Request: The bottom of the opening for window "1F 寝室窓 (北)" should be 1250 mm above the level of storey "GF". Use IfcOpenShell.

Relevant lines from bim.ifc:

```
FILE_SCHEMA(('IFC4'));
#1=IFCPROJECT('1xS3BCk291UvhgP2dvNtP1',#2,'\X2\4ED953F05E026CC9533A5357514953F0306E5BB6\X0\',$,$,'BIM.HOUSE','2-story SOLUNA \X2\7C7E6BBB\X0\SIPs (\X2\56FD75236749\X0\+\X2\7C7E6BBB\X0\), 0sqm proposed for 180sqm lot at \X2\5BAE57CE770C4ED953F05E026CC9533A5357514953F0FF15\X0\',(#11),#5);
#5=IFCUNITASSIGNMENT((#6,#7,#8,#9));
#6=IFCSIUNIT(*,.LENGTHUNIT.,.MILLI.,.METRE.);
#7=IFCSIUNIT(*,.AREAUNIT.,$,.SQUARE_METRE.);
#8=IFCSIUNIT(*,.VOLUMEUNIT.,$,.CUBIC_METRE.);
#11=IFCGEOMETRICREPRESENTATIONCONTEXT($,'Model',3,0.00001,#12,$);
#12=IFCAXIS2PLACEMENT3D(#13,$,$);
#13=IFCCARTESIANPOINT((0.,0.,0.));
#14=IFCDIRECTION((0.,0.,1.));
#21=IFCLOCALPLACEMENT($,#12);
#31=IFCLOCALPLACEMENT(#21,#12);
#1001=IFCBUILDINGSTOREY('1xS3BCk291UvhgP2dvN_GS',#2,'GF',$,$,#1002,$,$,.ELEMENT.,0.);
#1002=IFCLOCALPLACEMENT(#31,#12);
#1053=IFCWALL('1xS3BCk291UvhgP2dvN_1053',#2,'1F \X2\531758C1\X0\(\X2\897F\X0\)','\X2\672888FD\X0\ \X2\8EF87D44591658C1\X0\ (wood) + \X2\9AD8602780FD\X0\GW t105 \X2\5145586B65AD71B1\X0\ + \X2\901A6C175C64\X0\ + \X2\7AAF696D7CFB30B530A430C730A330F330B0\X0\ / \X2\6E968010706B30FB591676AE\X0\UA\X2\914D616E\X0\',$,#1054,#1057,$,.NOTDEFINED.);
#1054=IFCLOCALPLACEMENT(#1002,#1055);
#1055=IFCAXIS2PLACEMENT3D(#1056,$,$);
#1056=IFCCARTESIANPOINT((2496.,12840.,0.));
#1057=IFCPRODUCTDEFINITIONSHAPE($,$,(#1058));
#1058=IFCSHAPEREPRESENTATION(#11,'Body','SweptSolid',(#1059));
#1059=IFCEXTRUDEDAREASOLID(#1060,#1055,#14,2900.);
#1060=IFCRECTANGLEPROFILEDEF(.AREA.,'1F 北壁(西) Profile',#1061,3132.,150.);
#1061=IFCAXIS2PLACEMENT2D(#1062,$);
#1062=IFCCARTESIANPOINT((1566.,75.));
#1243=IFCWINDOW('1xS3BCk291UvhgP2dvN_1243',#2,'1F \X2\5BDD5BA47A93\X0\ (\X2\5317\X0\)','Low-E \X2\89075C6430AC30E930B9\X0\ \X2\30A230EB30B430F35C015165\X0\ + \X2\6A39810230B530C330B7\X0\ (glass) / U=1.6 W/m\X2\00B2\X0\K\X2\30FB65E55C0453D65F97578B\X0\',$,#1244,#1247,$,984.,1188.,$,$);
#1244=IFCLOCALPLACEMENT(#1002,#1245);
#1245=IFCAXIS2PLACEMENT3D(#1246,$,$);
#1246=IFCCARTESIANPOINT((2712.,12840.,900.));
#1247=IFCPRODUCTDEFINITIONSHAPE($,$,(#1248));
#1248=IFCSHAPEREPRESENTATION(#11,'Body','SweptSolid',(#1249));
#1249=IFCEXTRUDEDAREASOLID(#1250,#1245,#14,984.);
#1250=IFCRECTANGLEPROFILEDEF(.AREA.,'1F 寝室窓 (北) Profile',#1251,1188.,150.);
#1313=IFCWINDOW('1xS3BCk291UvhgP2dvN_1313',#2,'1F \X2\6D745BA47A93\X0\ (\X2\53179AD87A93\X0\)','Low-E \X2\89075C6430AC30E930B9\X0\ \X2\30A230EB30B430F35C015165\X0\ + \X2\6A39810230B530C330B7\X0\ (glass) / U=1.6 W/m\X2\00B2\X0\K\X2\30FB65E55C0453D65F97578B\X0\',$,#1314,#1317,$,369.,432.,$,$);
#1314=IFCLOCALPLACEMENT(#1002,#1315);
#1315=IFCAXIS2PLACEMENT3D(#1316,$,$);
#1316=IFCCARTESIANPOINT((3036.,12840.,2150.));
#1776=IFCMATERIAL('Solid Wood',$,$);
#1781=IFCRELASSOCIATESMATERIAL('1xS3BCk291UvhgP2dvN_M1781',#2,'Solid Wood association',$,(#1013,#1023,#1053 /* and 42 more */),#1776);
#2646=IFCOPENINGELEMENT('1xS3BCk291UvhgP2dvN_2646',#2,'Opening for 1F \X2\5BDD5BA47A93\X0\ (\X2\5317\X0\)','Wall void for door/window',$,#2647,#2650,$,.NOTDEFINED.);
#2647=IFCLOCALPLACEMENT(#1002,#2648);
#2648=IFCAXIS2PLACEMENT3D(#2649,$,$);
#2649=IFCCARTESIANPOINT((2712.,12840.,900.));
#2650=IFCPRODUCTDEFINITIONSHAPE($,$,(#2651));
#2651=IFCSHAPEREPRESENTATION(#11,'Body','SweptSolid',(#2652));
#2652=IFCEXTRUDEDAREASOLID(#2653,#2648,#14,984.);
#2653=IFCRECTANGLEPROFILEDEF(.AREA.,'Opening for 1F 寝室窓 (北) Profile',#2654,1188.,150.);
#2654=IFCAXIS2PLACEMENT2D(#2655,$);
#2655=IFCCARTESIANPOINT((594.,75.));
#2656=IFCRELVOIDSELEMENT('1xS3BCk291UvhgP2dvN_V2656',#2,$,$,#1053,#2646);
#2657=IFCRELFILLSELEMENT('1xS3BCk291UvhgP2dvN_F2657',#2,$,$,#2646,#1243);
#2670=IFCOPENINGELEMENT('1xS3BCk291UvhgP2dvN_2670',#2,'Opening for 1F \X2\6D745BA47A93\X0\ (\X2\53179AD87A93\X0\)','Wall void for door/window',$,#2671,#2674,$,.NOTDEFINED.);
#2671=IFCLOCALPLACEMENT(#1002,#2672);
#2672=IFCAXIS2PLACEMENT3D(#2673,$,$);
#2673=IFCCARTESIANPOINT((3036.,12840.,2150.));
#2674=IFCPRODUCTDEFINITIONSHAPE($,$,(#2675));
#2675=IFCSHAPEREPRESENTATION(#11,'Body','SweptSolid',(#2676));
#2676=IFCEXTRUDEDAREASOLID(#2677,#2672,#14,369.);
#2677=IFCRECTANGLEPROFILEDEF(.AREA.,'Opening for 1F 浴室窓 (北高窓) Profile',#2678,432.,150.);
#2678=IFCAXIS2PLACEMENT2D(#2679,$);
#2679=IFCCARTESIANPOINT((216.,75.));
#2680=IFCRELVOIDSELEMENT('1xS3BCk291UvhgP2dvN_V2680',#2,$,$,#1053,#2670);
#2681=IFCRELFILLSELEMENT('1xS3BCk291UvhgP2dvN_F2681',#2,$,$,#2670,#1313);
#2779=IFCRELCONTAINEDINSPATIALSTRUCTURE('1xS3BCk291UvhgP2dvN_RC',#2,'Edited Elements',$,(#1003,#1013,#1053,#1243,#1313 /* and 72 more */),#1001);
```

```python
import numpy as np
import ifcopenshell
import ifcopenshell.api.geometry
import ifcopenshell.geom
import ifcopenshell.util.element
import ifcopenshell.util.placement
import ifcopenshell.util.shape
import ifcopenshell.util.unit

model = ifcopenshell.open("bim.ifc")
unit_scale = ifcopenshell.util.unit.calculate_unit_scale(model)

window = model.by_guid("1xS3BCk291UvhgP2dvN_1243")
opening = window.FillsVoids[0].RelatingOpeningElement
storey = ifcopenshell.util.element.get_container(window, ifc_class="IfcBuildingStorey")
level = ifcopenshell.util.placement.get_local_placement(storey.ObjectPlacement)[2, 3]

# The opening's origin need not be at the sill, so measure its lowest point.
shape = ifcopenshell.geom.create_shape(ifcopenshell.geom.settings(), opening)
bottom = ifcopenshell.util.shape.get_shape_bottom_elevation(shape, shape.geometry) / unit_scale
dz = level + 1250.0 - bottom

shift = np.array([0.0, 0.0, dz])
# The window is not placed relative to its opening, so move both.
for product in (opening, window):
    matrix = ifcopenshell.util.placement.get_local_placement(product.ObjectPlacement)
    matrix[:3, 3] += shift
    ifcopenshell.api.geometry.edit_object_placement(model, product=product, matrix=matrix, is_si=False)

print(f"moved by {dz * unit_scale:+.3f} m")

model.write("bim-out.ifc")
```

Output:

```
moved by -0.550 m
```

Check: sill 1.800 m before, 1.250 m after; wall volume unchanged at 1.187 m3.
